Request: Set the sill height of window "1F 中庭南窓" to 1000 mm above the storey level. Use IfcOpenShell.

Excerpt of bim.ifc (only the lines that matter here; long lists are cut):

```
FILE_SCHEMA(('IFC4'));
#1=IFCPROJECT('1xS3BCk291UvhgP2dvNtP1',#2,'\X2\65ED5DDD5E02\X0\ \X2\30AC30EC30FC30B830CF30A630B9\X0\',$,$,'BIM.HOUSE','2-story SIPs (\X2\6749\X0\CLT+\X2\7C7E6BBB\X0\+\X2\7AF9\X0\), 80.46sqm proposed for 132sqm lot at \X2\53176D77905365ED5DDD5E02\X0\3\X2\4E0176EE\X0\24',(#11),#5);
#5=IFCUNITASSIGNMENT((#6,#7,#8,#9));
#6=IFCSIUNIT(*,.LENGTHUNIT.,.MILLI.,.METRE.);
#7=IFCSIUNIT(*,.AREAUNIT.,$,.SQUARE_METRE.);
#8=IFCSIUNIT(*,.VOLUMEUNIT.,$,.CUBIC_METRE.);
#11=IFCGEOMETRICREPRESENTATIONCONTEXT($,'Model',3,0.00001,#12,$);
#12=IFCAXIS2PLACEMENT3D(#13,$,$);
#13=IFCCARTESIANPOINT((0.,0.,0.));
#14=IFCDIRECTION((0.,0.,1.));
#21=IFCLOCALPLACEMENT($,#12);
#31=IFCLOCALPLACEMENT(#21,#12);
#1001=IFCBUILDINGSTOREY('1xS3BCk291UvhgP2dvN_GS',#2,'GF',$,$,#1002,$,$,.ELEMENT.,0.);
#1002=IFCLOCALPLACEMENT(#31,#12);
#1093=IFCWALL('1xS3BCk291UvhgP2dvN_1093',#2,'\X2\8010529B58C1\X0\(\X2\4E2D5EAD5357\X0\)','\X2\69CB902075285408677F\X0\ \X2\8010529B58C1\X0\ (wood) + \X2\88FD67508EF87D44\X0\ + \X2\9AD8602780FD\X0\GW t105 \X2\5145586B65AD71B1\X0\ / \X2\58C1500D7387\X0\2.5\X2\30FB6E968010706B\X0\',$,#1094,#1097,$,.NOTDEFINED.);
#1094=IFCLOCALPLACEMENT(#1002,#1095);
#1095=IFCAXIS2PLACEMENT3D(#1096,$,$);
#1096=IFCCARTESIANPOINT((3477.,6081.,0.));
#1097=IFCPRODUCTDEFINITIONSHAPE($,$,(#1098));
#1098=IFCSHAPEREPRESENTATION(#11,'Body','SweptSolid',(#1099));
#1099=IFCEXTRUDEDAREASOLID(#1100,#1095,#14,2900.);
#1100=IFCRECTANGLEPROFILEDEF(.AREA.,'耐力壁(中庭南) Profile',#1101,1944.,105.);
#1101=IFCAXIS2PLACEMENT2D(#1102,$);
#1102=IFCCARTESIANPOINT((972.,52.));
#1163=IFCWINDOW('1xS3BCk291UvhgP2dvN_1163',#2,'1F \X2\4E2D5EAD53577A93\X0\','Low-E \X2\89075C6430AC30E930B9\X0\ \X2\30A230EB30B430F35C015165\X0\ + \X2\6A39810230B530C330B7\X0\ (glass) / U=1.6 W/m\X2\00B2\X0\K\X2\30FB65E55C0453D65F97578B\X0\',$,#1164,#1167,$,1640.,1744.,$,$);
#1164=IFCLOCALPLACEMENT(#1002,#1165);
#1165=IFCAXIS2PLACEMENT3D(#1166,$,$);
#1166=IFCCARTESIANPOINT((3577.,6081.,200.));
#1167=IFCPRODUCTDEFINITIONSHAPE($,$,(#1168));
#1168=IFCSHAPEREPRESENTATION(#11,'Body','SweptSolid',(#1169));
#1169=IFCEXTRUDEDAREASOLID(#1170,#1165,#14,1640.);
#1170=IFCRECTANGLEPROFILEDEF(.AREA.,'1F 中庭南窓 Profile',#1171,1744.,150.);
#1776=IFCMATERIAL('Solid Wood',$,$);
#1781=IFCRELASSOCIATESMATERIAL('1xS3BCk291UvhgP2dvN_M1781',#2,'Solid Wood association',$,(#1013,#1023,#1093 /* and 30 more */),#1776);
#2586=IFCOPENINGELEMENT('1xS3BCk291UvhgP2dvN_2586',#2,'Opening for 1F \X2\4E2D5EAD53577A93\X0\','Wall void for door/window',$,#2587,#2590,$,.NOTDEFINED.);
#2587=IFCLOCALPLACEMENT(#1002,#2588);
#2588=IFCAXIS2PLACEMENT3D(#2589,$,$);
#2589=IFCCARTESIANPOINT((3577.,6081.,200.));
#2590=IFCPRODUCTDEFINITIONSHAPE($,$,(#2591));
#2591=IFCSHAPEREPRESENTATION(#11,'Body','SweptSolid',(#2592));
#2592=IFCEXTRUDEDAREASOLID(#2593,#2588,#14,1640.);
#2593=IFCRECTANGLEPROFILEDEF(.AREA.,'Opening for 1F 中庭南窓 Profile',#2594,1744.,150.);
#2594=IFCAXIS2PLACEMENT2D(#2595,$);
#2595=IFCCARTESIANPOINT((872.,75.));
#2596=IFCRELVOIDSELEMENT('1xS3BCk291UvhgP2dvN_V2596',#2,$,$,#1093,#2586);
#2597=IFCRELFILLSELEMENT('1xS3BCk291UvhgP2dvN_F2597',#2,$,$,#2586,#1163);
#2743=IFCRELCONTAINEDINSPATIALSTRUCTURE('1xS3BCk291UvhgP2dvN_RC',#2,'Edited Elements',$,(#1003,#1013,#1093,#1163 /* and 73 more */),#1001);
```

```python
import numpy as np
import ifcopenshell
import ifcopenshell.api.geometry
import ifcopenshell.geom
import ifcopenshell.util.element
import ifcopenshell.util.placement
import ifcopenshell.util.shape
import ifcopenshell.util.unit

model = ifcopenshell.open("bim.ifc")
unit_scale = ifcopenshell.util.unit.calculate_unit_scale(model)

window = model.by_id(1163)
opening = window.FillsVoids[0].RelatingOpeningElement
storey = ifcopenshell.util.element.get_container(window, ifc_class="IfcBuildingStorey")
level = ifcopenshell.util.placement.get_local_placement(storey.ObjectPlacement)[2, 3]

# The opening's origin need not be at the sill, so measure its lowest point.
shape = ifcopenshell.geom.create_shape(ifcopenshell.geom.settings(), opening)
bottom = ifcopenshell.util.shape.get_shape_bottom_elevation(shape, shape.geometry) / unit_scale
dz = level + 1 / unit_scale - bottom

shift = np.array([0.0, 0.0, dz])
# The window is not placed relative to its opening, so move both.
for product in (opening, window):
    matrix = ifcopenshell.util.placement.get_local_placement(product.ObjectPlacement)
    matrix[:3, 3] += shift
    ifcopenshell.api.geometry.edit_object_placement(model, product=product, matrix=matrix, is_si=False)

print(f"moved by {dz * unit_scale:+.3f} m")

model.write("bim_updated.ifc")
```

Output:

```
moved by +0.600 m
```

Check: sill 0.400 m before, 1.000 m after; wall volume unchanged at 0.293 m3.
